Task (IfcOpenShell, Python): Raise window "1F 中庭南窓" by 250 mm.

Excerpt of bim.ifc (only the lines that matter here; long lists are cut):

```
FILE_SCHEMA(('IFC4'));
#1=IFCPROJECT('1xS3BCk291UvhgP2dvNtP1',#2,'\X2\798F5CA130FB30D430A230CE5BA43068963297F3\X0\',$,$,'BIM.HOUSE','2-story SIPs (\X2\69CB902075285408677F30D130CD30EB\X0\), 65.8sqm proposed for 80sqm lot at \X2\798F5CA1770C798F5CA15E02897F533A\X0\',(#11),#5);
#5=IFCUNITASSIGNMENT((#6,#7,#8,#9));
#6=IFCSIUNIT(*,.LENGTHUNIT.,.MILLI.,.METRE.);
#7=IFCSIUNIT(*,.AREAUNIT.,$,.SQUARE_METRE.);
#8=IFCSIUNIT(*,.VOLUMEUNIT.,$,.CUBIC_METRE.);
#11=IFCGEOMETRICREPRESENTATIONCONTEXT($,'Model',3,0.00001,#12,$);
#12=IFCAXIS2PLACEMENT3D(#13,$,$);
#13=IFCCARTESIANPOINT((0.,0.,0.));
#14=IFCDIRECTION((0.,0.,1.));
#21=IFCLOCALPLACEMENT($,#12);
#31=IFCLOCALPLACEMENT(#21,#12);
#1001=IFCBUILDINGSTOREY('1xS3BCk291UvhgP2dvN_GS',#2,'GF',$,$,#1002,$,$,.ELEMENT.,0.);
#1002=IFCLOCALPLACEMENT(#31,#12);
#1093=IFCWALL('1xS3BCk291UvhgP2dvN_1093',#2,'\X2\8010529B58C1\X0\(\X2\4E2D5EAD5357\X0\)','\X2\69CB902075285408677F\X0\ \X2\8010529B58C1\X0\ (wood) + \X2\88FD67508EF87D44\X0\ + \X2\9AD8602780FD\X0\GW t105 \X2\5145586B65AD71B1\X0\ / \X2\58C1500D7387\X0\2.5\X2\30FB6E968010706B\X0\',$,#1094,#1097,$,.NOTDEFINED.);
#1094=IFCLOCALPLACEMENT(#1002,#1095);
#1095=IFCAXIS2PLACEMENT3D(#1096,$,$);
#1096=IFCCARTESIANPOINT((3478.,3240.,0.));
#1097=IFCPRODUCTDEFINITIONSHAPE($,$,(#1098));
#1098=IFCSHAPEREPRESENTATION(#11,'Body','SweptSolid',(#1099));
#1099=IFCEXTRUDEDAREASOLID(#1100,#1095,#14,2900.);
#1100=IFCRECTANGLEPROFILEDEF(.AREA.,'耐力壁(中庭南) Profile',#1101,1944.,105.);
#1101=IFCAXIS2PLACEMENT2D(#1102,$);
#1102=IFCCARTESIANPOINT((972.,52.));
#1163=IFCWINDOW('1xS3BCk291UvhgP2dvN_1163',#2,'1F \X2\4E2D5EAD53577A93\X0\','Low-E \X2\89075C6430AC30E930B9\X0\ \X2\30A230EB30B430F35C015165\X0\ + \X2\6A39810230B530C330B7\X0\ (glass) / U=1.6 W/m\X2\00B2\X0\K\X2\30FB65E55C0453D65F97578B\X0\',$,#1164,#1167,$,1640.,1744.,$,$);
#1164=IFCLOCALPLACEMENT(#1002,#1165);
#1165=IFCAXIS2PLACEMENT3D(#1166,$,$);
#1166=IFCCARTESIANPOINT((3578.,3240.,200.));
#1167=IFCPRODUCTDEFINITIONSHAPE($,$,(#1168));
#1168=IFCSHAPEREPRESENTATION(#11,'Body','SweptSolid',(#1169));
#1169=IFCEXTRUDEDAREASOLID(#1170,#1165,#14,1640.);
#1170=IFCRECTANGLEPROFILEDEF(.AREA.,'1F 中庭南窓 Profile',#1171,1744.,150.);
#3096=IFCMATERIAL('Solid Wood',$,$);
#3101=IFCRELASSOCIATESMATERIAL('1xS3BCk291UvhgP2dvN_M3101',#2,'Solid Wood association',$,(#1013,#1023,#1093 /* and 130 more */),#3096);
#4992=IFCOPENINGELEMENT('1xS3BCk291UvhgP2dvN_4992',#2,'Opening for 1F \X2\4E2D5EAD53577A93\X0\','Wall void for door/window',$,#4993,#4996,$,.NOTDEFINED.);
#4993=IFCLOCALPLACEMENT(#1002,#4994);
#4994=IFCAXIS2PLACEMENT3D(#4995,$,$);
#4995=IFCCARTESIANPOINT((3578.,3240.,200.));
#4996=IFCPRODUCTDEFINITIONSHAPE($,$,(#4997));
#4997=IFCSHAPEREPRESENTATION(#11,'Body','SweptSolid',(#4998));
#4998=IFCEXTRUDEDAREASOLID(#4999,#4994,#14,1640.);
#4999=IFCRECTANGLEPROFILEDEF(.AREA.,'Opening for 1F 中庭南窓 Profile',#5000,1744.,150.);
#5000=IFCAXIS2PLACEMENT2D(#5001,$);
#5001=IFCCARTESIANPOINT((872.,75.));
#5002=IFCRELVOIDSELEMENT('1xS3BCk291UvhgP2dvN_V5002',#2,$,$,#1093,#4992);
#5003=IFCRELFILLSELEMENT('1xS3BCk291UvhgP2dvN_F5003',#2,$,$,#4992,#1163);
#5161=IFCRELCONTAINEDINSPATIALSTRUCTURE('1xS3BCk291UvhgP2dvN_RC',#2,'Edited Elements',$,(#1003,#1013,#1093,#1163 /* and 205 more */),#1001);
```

```python
import numpy as np
import ifcopenshell
import ifcopenshell.api.geometry
import ifcopenshell.util.placement
import ifcopenshell.util.unit

model = ifcopenshell.open("bim.ifc")
unit_scale = ifcopenshell.util.unit.calculate_unit_scale(model)

window = model.by_guid("1xS3BCk291UvhgP2dvN_1163")
opening = window.FillsVoids[0].RelatingOpeningElement
dz = 0.25 / unit_scale

shift = np.array([0.0, 0.0, dz])
# The window is not placed relative to its opening, so move both.
for product in (opening, window):
    matrix = ifcopenshell.util.placement.get_local_placement(product.ObjectPlacement)
    matrix[:3, 3] += shift
    ifcopenshell.api.geometry.edit_object_placement(model, product=product, matrix=matrix, is_si=False)

print(f"moved by {dz * unit_scale:+.3f} m")

model.write("bim_v2.ifc")
```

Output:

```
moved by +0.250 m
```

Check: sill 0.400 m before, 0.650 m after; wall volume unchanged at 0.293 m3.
